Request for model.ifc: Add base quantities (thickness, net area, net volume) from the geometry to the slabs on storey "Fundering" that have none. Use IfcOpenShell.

First a look at what the model holds.

```python
import ifcopenshell
import ifcopenshell.util.element
import ifcopenshell.util.unit

model = ifcopenshell.open("model.ifc")
print(model.schema)
for unit_type in ("LENGTHUNIT", "AREAUNIT", "VOLUMEUNIT"):
    print(unit_type, ifcopenshell.util.unit.calculate_unit_scale(model, unit_type))
storey = next(s for s in model.by_type("IfcBuildingStorey") if s.Name == "Fundering")
slabs = [e for e in ifcopenshell.util.element.get_decomposition(storey) if e.is_a("IfcSlab")]
for e in sorted(slabs, key=lambda e: e.id()):
    print(e.id(), e.is_a(), e.Name, list(ifcopenshell.util.element.get_psets(e, qtos_only=True)), sep=" | ")
```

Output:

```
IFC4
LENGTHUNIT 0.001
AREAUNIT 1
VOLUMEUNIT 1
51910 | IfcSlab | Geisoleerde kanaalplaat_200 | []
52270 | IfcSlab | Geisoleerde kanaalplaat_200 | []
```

```python
import ifcopenshell
import ifcopenshell.api.pset
import ifcopenshell.geom
import ifcopenshell.util.element
import ifcopenshell.util.shape
import ifcopenshell.util.unit

model = ifcopenshell.open("model.ifc")
unit_scale = ifcopenshell.util.unit.calculate_unit_scale(model)
area_scale = ifcopenshell.util.unit.calculate_unit_scale(model, "AREAUNIT")
volume_scale = ifcopenshell.util.unit.calculate_unit_scale(model, "VOLUMEUNIT")
settings = ifcopenshell.geom.settings()

storey = next(s for s in model.by_type("IfcBuildingStorey") if s.Name == "Fundering")
slabs = [e for e in ifcopenshell.util.element.get_decomposition(storey) if e.is_a("IfcSlab")]

for e in sorted(slabs, key=lambda e: e.id()):
    if ifcopenshell.util.element.get_psets(e, qtos_only=True, should_inherit=False):
        continue
    # Geometry comes back in metres, in the element's own axes.
    shape = ifcopenshell.geom.create_shape(settings, e)
    values = {
        "Width": ifcopenshell.util.shape.get_z(shape.geometry) / unit_scale,
        "NetArea": ifcopenshell.util.shape.get_footprint_area(shape.geometry) / area_scale,
        "NetVolume": ifcopenshell.util.shape.get_volume(shape.geometry) / volume_scale,
    }
    qto = ifcopenshell.api.pset.add_qto(model, product=e, name="Qto_SlabBaseQuantities")
    ifcopenshell.api.pset.edit_qto(model, qto=qto, properties=values)
    print(e.id(), {k: round(v, 3) for k, v in values.items()})

model.write("model-out.ifc")
```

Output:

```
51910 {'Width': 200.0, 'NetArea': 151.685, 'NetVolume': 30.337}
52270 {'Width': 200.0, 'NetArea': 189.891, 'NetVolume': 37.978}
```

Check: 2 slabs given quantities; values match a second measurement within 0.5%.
